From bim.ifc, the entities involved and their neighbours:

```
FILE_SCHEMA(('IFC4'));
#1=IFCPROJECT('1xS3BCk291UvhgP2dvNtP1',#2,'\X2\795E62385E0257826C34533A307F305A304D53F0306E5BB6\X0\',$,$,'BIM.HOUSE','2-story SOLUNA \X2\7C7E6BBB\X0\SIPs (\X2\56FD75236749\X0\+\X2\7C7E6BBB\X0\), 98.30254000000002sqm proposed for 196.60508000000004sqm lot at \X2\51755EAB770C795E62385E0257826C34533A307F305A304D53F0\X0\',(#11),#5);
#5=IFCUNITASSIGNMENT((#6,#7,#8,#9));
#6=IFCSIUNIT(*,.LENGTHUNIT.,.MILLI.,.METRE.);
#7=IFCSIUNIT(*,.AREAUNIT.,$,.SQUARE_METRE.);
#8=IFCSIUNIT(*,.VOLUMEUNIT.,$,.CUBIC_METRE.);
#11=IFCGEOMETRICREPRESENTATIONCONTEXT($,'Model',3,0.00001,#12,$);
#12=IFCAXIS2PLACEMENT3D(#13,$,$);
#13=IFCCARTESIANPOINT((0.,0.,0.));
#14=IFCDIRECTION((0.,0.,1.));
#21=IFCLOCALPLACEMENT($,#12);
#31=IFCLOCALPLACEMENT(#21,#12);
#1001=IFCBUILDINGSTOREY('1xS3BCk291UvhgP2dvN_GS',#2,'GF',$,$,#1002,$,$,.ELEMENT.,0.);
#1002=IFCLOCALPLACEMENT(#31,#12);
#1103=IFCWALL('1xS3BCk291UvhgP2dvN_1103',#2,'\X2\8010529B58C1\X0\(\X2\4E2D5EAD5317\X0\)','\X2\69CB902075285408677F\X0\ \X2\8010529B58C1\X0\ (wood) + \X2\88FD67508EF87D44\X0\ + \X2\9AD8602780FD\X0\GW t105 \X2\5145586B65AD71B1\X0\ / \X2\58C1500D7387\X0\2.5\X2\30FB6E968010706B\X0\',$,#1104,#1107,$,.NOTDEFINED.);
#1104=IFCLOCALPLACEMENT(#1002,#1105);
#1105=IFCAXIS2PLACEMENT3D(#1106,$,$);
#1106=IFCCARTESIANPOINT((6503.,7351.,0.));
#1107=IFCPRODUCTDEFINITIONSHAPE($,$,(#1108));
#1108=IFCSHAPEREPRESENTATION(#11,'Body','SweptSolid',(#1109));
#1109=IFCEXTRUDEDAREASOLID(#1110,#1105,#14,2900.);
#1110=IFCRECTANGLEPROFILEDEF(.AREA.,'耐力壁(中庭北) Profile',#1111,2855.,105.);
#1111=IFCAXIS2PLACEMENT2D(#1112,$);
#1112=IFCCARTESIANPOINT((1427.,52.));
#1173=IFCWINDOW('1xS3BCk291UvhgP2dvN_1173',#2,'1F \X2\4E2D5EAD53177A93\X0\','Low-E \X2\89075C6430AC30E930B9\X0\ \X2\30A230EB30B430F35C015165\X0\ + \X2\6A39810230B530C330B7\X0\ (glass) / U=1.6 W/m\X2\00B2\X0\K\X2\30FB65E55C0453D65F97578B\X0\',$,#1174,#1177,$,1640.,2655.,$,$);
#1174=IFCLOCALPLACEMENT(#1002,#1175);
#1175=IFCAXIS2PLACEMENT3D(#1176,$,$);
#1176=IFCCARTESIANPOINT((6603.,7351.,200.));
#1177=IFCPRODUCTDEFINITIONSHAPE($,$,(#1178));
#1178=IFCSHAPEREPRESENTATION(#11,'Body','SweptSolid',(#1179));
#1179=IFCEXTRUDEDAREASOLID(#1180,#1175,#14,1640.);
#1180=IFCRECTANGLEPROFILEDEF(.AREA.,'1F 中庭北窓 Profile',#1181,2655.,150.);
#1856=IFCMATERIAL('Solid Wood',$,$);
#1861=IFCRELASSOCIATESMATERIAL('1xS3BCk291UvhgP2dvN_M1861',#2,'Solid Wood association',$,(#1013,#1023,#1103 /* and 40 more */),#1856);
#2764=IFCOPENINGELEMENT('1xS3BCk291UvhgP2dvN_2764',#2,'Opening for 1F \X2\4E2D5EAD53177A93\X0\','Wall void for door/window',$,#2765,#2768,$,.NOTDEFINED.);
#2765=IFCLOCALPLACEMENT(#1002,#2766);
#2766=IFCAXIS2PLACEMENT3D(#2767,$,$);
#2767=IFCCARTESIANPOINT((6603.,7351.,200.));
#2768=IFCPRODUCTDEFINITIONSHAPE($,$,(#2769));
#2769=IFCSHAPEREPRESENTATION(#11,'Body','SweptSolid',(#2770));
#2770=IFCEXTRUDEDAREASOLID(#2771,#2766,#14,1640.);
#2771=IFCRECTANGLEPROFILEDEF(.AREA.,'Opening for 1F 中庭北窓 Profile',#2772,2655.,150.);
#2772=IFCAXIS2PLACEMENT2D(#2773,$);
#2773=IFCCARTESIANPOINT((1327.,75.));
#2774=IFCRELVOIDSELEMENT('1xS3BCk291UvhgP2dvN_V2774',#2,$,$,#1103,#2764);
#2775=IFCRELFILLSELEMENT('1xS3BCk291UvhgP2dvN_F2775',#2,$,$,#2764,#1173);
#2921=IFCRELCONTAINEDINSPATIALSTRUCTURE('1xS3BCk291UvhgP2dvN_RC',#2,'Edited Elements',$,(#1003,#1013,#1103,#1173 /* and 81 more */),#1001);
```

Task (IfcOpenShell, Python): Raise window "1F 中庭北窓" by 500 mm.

```python
import numpy as np
import ifcopenshell
import ifcopenshell.api.geometry
import ifcopenshell.util.placement
import ifcopenshell.util.unit

model = ifcopenshell.open("bim.ifc")
unit_scale = ifcopenshell.util.unit.calculate_unit_scale(model)

window = model.by_id(1173)
opening = window.FillsVoids[0].RelatingOpeningElement
dz = 0.5 / unit_scale

shift = np.array([0.0, 0.0, dz])
# The window is not placed relative to its opening, so move both.
for product in (opening, window):
    matrix = ifcopenshell.util.placement.get_local_placement(product.ObjectPlacement)
    matrix[:3, 3] += shift
    ifcopenshell.api.geometry.edit_object_placement(model, product=product, matrix=matrix, is_si=False)

print(f"moved by {dz * unit_scale:+.3f} m")

model.write("bim_rev.ifc")
```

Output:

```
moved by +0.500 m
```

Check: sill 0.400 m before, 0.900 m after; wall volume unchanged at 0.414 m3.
